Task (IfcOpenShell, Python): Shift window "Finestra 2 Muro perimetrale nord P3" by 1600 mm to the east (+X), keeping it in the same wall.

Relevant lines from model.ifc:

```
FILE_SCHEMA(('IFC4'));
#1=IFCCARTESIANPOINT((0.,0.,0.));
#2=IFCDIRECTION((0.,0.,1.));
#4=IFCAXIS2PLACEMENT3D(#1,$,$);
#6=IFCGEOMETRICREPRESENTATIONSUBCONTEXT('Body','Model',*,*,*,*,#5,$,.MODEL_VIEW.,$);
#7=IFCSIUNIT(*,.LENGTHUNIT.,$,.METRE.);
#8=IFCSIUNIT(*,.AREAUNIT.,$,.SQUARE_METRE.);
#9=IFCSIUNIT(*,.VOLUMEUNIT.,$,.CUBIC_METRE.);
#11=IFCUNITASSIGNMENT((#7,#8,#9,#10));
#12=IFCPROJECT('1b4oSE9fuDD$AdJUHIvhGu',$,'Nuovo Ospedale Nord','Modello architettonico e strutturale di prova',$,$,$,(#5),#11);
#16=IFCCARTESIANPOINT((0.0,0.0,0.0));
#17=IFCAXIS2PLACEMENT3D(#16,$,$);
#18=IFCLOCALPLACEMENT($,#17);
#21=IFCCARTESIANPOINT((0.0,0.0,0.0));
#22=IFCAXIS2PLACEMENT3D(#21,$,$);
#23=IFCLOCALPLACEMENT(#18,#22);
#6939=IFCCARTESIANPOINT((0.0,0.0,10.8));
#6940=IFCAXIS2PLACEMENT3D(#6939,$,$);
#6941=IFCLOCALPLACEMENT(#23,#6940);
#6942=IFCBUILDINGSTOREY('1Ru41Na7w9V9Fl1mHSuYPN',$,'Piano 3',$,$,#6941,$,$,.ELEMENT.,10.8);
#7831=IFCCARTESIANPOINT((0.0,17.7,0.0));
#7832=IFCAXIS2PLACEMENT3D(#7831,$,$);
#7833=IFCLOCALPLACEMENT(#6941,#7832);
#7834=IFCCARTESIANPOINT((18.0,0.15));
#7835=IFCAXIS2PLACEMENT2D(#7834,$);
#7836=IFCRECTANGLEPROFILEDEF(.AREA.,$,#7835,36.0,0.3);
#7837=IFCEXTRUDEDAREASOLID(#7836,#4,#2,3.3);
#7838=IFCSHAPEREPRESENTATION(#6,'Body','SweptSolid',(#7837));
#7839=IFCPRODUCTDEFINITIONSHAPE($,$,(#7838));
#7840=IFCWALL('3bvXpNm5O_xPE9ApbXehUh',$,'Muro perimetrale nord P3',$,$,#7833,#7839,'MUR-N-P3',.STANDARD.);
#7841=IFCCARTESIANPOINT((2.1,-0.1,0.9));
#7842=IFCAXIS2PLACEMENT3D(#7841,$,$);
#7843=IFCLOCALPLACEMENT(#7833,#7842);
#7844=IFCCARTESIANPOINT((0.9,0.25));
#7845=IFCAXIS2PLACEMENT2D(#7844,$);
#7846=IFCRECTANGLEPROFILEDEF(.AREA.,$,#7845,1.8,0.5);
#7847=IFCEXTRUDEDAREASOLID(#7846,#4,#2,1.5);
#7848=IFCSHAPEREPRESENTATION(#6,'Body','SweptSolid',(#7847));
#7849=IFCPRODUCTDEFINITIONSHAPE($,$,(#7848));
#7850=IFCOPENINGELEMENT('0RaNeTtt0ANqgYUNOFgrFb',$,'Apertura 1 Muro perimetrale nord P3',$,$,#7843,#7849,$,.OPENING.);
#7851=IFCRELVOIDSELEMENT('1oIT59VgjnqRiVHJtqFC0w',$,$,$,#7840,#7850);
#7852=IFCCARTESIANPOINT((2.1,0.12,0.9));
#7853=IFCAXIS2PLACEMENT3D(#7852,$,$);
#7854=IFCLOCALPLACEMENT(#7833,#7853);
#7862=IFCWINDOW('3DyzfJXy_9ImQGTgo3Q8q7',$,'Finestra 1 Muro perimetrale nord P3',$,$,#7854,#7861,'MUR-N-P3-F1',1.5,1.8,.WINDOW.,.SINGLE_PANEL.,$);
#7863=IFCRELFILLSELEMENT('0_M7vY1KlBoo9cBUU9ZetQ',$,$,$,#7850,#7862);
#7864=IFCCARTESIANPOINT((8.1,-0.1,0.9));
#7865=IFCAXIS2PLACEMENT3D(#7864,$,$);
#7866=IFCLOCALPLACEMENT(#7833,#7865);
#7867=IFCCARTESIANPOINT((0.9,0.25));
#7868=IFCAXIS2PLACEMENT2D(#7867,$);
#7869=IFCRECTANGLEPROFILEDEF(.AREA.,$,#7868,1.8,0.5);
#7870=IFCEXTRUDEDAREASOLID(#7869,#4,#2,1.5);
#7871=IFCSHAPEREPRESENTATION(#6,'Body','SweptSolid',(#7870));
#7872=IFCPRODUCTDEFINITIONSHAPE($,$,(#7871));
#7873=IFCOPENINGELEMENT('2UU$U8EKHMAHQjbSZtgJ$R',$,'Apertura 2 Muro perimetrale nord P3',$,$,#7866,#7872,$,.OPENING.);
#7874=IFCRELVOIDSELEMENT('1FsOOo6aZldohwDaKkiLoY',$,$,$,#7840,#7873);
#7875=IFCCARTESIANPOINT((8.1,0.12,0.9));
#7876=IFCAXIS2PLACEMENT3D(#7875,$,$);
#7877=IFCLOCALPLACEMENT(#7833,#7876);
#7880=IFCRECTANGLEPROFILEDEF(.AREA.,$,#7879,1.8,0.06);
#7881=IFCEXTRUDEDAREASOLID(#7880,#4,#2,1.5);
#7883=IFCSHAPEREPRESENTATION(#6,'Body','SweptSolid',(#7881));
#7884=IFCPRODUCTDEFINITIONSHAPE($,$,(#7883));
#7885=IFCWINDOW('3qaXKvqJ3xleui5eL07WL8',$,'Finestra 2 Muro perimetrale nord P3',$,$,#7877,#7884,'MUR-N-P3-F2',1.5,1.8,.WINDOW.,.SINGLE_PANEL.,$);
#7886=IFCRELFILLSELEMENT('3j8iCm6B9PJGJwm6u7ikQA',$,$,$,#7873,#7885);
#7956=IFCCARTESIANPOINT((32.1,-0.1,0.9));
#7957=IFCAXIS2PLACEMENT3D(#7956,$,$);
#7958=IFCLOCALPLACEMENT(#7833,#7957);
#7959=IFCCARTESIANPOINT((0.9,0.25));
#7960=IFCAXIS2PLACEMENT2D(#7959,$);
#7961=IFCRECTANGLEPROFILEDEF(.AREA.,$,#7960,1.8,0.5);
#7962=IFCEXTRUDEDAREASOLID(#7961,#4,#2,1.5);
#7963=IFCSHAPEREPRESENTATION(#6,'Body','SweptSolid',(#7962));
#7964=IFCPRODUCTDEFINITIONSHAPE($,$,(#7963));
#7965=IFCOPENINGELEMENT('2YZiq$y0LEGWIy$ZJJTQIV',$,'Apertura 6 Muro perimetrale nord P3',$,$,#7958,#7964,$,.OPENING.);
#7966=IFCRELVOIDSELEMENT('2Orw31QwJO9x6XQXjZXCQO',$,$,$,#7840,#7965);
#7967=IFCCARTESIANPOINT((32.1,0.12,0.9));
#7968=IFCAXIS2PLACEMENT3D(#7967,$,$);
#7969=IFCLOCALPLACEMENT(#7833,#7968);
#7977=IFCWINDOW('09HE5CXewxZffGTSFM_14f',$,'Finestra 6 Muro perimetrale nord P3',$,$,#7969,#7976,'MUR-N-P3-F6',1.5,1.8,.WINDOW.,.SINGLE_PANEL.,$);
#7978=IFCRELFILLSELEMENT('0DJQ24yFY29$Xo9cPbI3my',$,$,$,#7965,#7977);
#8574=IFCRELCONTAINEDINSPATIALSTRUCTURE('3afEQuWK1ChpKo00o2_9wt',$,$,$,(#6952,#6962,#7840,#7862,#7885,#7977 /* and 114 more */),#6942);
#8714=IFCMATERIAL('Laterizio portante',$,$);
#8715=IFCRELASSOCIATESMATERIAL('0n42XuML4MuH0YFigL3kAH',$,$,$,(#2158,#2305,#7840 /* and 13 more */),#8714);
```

```python
import ifcopenshell
import ifcopenshell.api.geometry
import ifcopenshell.util.placement
import ifcopenshell.util.unit

model = ifcopenshell.open("model.ifc")
unit_scale = ifcopenshell.util.unit.calculate_unit_scale(model)

window = model.by_guid("3qaXKvqJ3xleui5eL07WL8")
opening = window.FillsVoids[0].RelatingOpeningElement
wall = opening.VoidsElements[0].RelatingBuildingElement

wall_matrix = ifcopenshell.util.placement.get_local_placement(wall.ObjectPlacement)
shift = wall_matrix[:3, 0] * 1.6 / unit_scale
before = ifcopenshell.util.placement.get_local_placement(window.ObjectPlacement)[:3, 3].copy()

# The window is not placed relative to its opening, so move both.
for product in (opening, window):
    matrix = ifcopenshell.util.placement.get_local_placement(product.ObjectPlacement)
    matrix[:3, 3] += shift
    ifcopenshell.api.geometry.edit_object_placement(model, product=product, matrix=matrix, is_si=False)

after = ifcopenshell.util.placement.get_local_placement(window.ObjectPlacement)[:3, 3]
print("window moved by", (after - before).round(3) + 0.0)

model.write("model_updated.ifc")
```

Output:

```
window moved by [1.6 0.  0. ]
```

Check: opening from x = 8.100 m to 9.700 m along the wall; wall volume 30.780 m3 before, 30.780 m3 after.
